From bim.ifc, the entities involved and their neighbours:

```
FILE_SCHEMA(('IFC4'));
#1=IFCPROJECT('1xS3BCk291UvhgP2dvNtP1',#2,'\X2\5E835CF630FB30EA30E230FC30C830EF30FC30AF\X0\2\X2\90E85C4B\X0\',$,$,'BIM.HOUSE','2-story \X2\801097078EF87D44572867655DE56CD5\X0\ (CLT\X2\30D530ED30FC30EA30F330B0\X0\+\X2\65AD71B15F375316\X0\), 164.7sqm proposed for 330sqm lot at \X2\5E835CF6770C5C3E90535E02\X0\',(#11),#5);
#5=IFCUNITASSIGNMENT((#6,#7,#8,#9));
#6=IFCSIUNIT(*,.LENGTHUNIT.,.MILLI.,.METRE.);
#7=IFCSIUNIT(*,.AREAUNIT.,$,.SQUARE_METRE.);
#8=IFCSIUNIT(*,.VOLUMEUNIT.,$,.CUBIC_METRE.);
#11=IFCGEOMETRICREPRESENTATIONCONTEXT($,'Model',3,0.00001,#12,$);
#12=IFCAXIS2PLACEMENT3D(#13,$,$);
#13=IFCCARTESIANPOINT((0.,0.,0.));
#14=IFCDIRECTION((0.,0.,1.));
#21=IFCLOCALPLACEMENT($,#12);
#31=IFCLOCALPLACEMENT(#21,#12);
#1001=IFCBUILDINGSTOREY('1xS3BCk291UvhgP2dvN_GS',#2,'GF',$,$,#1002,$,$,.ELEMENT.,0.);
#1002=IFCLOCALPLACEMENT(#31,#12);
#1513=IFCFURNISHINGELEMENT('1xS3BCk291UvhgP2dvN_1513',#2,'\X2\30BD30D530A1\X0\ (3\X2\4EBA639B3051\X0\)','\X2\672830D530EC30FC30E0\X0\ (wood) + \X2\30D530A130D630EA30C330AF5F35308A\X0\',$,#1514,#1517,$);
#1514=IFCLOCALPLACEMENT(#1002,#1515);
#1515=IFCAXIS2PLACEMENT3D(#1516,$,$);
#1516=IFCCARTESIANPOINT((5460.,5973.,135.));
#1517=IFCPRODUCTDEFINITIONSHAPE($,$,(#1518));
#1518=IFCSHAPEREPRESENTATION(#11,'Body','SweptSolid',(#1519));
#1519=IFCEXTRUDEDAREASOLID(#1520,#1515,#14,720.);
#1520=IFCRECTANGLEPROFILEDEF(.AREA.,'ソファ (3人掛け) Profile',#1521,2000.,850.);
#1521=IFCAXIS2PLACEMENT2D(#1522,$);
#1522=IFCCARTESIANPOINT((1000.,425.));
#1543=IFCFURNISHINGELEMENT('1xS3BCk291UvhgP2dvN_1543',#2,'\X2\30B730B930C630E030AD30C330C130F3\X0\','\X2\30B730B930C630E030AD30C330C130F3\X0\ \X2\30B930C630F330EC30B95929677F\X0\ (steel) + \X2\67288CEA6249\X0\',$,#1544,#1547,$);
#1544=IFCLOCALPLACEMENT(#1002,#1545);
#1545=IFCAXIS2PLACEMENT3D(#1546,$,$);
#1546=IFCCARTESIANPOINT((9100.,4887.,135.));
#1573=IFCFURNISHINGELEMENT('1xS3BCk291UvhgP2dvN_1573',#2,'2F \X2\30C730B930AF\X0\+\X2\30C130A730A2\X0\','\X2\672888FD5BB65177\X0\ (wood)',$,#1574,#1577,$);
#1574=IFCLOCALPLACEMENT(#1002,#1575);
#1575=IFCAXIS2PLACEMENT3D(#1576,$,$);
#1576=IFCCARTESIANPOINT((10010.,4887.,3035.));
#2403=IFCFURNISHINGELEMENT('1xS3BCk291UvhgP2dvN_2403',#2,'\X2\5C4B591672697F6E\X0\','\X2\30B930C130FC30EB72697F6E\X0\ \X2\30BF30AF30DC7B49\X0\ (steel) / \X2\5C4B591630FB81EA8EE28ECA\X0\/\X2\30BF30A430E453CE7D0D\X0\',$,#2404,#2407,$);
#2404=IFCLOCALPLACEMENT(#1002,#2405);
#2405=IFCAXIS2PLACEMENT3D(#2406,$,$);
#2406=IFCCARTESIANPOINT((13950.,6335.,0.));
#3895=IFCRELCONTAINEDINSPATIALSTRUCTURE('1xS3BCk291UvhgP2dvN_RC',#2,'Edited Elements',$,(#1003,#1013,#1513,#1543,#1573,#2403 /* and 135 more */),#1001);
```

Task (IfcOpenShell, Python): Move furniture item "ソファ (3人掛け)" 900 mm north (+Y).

```python
import ifcopenshell
import ifcopenshell.api.geometry
import ifcopenshell.util.placement

model = ifcopenshell.open("bim.ifc")

item = model.by_guid("1xS3BCk291UvhgP2dvN_1513")
matrix = ifcopenshell.util.placement.get_local_placement(item.ObjectPlacement)
matrix[1, 3] += 900.0
ifcopenshell.api.geometry.edit_object_placement(model, product=item, matrix=matrix, is_si=False)

print(ifcopenshell.util.placement.get_local_placement(item.ObjectPlacement).round(3) + 0.0)

model.write("bim_edited.ifc")
```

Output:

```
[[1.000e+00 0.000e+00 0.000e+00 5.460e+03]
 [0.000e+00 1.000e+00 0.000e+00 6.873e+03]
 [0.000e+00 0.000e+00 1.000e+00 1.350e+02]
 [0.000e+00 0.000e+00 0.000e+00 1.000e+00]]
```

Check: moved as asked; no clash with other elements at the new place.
